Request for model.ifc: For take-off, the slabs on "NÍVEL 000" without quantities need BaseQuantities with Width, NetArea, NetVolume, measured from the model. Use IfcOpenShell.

First a look at what the model holds.

```python
import ifcopenshell
import ifcopenshell.util.element
import ifcopenshell.util.unit

model = ifcopenshell.open("model.ifc")
print(model.schema)
for unit_type in ("LENGTHUNIT", "AREAUNIT", "VOLUMEUNIT"):
    print(unit_type, ifcopenshell.util.unit.calculate_unit_scale(model, unit_type))
storey = next(s for s in model.by_type("IfcBuildingStorey") if s.Name == "NÍVEL 000")
slabs = [e for e in ifcopenshell.util.element.get_decomposition(storey) if e.is_a("IfcSlab")]
for e in sorted(slabs, key=lambda e: e.id()):
    print(e.id(), e.is_a(), e.Name, list(ifcopenshell.util.element.get_psets(e, qtos_only=True)), sep=" | ")
```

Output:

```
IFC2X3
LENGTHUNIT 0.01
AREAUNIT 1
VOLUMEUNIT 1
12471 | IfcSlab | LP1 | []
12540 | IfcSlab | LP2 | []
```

```python
import ifcopenshell
import ifcopenshell.api.pset
import ifcopenshell.geom
import ifcopenshell.util.element
import ifcopenshell.util.shape
import ifcopenshell.util.unit

model = ifcopenshell.open("model.ifc")
unit_scale = ifcopenshell.util.unit.calculate_unit_scale(model)
area_scale = ifcopenshell.util.unit.calculate_unit_scale(model, "AREAUNIT")
volume_scale = ifcopenshell.util.unit.calculate_unit_scale(model, "VOLUMEUNIT")
settings = ifcopenshell.geom.settings()

storey = next(s for s in model.by_type("IfcBuildingStorey") if s.Name == "NÍVEL 000")
slabs = [e for e in ifcopenshell.util.element.get_decomposition(storey) if e.is_a("IfcSlab")]

for e in sorted(slabs, key=lambda e: e.id()):
    if ifcopenshell.util.element.get_psets(e, qtos_only=True, should_inherit=False):
        continue
    # Geometry comes back in metres, in the element's own axes.
    shape = ifcopenshell.geom.create_shape(settings, e)
    values = {
        "Width": ifcopenshell.util.shape.get_z(shape.geometry) / unit_scale,
        "NetArea": ifcopenshell.util.shape.get_footprint_area(shape.geometry) / area_scale,
        "NetVolume": ifcopenshell.util.shape.get_volume(shape.geometry) / volume_scale,
    }
    qto = ifcopenshell.api.pset.add_qto(model, product=e, name="BaseQuantities")
    ifcopenshell.api.pset.edit_qto(model, qto=qto, properties=values)
    print(e.id(), {k: round(v, 3) for k, v in values.items()})

model.write("model-out.ifc")
```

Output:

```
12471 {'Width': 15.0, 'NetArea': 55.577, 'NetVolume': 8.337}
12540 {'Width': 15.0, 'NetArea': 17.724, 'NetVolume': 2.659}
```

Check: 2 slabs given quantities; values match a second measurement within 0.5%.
